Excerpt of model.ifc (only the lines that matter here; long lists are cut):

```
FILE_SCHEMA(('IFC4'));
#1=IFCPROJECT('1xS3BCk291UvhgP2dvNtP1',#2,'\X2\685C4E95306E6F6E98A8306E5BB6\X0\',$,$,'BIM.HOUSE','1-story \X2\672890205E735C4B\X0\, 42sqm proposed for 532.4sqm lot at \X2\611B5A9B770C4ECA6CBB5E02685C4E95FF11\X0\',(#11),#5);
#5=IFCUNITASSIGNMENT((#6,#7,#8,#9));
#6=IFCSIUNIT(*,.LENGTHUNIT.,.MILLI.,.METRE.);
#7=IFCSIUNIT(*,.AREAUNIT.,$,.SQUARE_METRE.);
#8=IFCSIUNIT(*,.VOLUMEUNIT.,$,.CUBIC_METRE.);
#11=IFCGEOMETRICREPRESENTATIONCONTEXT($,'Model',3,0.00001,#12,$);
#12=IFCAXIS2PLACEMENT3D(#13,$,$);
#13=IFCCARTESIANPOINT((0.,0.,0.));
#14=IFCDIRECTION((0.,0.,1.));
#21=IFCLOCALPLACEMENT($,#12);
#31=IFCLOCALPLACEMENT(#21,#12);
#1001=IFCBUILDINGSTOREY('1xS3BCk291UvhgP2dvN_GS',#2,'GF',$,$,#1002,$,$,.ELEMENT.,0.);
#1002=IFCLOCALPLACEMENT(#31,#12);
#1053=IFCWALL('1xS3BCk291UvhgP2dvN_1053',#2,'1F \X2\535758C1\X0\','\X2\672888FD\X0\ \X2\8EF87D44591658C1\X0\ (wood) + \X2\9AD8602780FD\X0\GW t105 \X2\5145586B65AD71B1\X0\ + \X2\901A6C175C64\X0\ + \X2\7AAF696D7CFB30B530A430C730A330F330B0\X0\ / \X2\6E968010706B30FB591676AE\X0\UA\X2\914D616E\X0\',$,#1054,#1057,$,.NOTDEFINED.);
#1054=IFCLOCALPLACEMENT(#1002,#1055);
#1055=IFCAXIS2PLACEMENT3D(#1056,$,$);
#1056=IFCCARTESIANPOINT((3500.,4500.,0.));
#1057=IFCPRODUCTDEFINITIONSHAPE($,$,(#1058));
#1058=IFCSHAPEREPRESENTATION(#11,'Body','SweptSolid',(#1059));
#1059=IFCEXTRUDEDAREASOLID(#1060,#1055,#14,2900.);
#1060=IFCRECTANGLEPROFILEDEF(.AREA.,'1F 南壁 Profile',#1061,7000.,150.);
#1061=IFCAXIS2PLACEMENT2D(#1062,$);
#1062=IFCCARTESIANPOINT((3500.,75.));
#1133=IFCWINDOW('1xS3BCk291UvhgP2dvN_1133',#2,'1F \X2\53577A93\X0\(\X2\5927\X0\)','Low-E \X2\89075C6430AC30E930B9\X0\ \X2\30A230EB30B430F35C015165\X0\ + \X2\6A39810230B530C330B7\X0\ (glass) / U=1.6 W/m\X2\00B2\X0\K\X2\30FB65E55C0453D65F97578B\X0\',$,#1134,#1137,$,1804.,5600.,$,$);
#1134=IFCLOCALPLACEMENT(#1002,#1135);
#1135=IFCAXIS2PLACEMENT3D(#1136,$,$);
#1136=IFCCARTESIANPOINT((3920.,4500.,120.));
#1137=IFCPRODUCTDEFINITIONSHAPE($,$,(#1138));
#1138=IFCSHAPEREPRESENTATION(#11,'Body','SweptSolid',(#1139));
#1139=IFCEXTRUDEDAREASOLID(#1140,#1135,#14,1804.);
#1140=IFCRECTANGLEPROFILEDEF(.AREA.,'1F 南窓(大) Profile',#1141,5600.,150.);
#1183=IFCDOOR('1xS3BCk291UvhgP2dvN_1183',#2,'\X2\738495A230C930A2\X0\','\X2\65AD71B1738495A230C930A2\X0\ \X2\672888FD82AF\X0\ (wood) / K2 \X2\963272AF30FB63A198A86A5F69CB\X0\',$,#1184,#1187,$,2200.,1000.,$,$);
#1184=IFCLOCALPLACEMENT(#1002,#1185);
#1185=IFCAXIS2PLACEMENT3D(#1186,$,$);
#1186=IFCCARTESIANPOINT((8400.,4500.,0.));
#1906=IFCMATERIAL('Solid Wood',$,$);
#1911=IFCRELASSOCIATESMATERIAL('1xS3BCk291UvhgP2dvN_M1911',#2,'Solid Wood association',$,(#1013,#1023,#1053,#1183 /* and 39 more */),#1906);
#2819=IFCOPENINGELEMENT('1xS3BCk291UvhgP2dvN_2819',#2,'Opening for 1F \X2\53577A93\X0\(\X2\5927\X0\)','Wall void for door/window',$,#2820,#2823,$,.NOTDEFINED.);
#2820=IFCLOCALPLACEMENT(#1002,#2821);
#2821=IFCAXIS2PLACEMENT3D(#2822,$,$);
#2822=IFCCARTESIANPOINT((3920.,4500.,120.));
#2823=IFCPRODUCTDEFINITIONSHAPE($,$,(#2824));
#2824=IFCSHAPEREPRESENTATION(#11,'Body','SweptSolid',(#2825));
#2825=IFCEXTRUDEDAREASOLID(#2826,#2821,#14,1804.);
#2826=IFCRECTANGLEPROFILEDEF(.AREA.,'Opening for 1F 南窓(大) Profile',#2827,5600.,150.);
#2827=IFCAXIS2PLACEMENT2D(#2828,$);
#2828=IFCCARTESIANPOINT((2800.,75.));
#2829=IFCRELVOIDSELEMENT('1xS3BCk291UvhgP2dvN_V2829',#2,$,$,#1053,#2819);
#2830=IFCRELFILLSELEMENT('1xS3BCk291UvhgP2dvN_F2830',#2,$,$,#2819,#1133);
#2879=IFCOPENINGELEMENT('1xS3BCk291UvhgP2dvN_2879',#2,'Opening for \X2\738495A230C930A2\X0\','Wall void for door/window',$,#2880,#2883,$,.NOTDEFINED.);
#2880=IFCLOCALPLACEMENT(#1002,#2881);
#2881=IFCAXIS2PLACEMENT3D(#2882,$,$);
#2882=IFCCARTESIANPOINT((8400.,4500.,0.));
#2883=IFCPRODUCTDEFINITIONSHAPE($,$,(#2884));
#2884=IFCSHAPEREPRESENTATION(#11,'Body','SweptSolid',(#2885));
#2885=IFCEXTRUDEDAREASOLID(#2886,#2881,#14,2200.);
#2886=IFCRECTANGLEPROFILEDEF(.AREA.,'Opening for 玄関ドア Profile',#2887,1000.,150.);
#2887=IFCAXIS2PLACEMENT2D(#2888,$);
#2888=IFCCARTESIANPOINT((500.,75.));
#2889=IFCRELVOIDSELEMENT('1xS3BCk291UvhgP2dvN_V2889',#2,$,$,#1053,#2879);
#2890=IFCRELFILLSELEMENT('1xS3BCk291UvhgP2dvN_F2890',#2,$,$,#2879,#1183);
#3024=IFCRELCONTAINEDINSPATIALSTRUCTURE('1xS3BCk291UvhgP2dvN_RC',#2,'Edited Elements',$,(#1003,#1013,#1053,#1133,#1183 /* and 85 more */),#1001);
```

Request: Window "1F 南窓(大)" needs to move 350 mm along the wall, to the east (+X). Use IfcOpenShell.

```python
import ifcopenshell
import ifcopenshell.api.geometry
import ifcopenshell.util.placement
import ifcopenshell.util.unit

model = ifcopenshell.open("model.ifc")
unit_scale = ifcopenshell.util.unit.calculate_unit_scale(model)

window = model.by_id(1133)
opening = window.FillsVoids[0].RelatingOpeningElement
wall = opening.VoidsElements[0].RelatingBuildingElement

wall_matrix = ifcopenshell.util.placement.get_local_placement(wall.ObjectPlacement)
shift = wall_matrix[:3, 0] * 0.35 / unit_scale
before = ifcopenshell.util.placement.get_local_placement(window.ObjectPlacement)[:3, 3].copy()

# The window is not placed relative to its opening, so move both.
for product in (opening, window):
    matrix = ifcopenshell.util.placement.get_local_placement(product.ObjectPlacement)
    matrix[:3, 3] += shift
    ifcopenshell.api.geometry.edit_object_placement(model, product=product, matrix=matrix, is_si=False)

after = ifcopenshell.util.placement.get_local_placement(window.ObjectPlacement)[:3, 3]
print("window moved by", (after - before).round(3) + 0.0)

model.write("model_updated.ifc")
```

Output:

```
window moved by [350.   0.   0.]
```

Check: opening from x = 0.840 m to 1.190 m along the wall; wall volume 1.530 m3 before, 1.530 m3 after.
